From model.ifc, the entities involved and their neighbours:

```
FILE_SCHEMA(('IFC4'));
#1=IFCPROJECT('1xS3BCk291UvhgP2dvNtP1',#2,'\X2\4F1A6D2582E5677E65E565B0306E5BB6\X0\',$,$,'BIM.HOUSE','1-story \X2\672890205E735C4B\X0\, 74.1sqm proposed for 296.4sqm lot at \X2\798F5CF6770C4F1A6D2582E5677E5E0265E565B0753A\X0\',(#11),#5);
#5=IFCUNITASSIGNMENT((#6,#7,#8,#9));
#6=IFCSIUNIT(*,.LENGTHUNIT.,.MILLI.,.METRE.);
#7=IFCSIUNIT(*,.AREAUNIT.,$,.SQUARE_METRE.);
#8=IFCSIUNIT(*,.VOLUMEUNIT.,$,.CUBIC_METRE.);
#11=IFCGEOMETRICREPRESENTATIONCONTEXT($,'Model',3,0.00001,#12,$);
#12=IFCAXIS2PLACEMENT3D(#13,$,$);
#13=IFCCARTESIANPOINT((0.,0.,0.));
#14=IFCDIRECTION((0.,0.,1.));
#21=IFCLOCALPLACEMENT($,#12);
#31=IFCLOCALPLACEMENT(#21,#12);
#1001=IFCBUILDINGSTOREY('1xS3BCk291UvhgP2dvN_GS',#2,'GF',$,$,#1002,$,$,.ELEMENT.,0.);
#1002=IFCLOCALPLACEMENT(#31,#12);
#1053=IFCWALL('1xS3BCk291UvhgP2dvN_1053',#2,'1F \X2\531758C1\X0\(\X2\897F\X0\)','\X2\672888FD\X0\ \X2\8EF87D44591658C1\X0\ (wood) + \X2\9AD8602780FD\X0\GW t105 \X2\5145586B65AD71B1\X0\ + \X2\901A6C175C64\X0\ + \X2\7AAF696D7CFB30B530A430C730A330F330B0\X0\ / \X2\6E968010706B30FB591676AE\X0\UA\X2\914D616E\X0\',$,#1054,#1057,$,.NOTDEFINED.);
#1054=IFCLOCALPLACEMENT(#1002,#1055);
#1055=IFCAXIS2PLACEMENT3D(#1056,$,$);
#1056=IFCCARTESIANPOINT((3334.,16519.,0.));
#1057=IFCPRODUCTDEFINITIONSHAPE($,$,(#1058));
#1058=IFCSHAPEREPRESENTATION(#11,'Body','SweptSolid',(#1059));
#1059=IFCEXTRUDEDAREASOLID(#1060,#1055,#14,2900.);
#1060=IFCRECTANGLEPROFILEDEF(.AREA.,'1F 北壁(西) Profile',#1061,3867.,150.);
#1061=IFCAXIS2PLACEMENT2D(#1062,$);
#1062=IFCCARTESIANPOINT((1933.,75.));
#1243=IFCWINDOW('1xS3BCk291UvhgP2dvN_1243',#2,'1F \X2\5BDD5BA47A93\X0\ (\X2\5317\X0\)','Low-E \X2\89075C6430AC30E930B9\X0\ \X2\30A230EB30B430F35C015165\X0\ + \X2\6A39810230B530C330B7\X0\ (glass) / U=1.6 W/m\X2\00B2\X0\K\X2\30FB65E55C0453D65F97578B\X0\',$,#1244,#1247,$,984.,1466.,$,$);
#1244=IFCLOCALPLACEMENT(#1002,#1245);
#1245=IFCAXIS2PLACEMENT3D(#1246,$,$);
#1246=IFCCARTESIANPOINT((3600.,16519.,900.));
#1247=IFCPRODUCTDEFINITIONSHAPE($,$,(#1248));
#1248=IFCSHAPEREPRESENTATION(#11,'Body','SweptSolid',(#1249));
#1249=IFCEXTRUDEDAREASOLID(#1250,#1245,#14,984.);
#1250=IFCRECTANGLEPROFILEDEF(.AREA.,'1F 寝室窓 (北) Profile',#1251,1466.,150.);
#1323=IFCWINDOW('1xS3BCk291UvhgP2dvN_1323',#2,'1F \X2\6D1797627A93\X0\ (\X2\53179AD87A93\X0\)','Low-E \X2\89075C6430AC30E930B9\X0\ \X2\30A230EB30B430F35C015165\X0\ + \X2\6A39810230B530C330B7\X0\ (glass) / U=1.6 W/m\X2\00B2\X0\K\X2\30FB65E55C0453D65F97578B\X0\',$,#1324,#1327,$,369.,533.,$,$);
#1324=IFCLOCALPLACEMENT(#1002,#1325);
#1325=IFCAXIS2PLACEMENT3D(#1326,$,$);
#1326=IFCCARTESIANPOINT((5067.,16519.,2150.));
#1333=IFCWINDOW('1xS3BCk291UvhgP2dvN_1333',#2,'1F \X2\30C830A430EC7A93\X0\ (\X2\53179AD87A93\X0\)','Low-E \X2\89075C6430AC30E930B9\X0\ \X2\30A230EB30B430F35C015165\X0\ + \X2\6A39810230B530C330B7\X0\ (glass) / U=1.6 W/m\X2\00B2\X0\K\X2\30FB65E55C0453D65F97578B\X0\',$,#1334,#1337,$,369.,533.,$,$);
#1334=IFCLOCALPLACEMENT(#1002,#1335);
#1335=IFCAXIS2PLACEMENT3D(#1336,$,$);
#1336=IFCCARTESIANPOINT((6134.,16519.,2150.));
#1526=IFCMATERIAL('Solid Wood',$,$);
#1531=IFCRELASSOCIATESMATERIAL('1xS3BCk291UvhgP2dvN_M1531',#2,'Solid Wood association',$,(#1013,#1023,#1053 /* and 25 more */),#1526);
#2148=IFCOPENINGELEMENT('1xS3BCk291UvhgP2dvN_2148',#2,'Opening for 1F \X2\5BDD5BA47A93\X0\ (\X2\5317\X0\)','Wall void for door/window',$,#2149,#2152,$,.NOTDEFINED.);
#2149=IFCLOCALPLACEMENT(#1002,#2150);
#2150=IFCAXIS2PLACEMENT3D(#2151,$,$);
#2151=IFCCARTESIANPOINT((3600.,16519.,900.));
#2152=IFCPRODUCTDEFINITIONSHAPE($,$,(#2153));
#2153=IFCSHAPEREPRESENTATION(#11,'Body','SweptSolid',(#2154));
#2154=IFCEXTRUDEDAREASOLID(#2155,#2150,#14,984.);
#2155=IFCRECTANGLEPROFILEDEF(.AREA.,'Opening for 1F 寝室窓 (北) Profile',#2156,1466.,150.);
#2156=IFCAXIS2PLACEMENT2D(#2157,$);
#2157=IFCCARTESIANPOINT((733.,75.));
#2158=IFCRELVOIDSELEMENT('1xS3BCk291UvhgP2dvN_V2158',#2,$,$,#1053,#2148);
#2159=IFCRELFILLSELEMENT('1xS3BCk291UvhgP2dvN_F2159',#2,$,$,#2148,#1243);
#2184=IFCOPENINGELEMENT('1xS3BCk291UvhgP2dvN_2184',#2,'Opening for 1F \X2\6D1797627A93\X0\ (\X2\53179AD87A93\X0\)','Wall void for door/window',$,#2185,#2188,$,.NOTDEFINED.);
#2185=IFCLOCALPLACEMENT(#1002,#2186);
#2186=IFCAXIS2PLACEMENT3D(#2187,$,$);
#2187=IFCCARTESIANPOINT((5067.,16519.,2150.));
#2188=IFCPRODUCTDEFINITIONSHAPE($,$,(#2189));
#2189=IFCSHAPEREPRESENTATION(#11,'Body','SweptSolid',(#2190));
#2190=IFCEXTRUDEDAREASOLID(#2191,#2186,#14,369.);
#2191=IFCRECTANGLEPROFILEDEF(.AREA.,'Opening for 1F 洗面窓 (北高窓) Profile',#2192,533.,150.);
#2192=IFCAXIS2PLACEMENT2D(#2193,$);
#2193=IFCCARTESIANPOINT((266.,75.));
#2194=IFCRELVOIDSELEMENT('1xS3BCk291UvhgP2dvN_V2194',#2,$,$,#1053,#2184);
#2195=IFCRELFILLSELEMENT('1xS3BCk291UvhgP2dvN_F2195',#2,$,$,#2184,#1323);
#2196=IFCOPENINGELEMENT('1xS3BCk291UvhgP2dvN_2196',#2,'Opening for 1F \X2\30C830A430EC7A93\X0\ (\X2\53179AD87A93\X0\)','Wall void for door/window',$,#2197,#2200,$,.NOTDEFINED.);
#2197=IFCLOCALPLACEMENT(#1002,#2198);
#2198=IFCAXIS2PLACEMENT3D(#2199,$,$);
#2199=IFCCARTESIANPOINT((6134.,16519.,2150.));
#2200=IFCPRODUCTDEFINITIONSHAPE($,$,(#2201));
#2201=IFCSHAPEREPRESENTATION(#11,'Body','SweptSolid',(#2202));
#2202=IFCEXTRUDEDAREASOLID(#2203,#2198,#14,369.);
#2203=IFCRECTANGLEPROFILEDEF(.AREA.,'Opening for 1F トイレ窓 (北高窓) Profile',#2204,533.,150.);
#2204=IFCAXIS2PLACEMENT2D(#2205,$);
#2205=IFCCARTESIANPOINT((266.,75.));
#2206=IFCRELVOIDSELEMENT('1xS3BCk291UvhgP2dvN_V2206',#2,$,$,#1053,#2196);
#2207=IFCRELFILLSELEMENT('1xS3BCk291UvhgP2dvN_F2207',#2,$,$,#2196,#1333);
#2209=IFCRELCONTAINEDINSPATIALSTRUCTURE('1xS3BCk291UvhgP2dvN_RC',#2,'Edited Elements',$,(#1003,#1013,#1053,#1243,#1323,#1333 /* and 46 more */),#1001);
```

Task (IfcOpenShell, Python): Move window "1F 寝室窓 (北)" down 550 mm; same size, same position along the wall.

```python
import numpy as np
import ifcopenshell
import ifcopenshell.api.geometry
import ifcopenshell.util.placement
import ifcopenshell.util.unit

model = ifcopenshell.open("model.ifc")
unit_scale = ifcopenshell.util.unit.calculate_unit_scale(model)

window = model.by_guid("1xS3BCk291UvhgP2dvN_1243")
opening = window.FillsVoids[0].RelatingOpeningElement
dz = -0.55 / unit_scale

shift = np.array([0.0, 0.0, dz])
# The window is not placed relative to its opening, so move both.
for product in (opening, window):
    matrix = ifcopenshell.util.placement.get_local_placement(product.ObjectPlacement)
    matrix[:3, 3] += shift
    ifcopenshell.api.geometry.edit_object_placement(model, product=product, matrix=matrix, is_si=False)

print(f"moved by {dz * unit_scale:+.3f} m")

model.write("model_v2.ifc")
```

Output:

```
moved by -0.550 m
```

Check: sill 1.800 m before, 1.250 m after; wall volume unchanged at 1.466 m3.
